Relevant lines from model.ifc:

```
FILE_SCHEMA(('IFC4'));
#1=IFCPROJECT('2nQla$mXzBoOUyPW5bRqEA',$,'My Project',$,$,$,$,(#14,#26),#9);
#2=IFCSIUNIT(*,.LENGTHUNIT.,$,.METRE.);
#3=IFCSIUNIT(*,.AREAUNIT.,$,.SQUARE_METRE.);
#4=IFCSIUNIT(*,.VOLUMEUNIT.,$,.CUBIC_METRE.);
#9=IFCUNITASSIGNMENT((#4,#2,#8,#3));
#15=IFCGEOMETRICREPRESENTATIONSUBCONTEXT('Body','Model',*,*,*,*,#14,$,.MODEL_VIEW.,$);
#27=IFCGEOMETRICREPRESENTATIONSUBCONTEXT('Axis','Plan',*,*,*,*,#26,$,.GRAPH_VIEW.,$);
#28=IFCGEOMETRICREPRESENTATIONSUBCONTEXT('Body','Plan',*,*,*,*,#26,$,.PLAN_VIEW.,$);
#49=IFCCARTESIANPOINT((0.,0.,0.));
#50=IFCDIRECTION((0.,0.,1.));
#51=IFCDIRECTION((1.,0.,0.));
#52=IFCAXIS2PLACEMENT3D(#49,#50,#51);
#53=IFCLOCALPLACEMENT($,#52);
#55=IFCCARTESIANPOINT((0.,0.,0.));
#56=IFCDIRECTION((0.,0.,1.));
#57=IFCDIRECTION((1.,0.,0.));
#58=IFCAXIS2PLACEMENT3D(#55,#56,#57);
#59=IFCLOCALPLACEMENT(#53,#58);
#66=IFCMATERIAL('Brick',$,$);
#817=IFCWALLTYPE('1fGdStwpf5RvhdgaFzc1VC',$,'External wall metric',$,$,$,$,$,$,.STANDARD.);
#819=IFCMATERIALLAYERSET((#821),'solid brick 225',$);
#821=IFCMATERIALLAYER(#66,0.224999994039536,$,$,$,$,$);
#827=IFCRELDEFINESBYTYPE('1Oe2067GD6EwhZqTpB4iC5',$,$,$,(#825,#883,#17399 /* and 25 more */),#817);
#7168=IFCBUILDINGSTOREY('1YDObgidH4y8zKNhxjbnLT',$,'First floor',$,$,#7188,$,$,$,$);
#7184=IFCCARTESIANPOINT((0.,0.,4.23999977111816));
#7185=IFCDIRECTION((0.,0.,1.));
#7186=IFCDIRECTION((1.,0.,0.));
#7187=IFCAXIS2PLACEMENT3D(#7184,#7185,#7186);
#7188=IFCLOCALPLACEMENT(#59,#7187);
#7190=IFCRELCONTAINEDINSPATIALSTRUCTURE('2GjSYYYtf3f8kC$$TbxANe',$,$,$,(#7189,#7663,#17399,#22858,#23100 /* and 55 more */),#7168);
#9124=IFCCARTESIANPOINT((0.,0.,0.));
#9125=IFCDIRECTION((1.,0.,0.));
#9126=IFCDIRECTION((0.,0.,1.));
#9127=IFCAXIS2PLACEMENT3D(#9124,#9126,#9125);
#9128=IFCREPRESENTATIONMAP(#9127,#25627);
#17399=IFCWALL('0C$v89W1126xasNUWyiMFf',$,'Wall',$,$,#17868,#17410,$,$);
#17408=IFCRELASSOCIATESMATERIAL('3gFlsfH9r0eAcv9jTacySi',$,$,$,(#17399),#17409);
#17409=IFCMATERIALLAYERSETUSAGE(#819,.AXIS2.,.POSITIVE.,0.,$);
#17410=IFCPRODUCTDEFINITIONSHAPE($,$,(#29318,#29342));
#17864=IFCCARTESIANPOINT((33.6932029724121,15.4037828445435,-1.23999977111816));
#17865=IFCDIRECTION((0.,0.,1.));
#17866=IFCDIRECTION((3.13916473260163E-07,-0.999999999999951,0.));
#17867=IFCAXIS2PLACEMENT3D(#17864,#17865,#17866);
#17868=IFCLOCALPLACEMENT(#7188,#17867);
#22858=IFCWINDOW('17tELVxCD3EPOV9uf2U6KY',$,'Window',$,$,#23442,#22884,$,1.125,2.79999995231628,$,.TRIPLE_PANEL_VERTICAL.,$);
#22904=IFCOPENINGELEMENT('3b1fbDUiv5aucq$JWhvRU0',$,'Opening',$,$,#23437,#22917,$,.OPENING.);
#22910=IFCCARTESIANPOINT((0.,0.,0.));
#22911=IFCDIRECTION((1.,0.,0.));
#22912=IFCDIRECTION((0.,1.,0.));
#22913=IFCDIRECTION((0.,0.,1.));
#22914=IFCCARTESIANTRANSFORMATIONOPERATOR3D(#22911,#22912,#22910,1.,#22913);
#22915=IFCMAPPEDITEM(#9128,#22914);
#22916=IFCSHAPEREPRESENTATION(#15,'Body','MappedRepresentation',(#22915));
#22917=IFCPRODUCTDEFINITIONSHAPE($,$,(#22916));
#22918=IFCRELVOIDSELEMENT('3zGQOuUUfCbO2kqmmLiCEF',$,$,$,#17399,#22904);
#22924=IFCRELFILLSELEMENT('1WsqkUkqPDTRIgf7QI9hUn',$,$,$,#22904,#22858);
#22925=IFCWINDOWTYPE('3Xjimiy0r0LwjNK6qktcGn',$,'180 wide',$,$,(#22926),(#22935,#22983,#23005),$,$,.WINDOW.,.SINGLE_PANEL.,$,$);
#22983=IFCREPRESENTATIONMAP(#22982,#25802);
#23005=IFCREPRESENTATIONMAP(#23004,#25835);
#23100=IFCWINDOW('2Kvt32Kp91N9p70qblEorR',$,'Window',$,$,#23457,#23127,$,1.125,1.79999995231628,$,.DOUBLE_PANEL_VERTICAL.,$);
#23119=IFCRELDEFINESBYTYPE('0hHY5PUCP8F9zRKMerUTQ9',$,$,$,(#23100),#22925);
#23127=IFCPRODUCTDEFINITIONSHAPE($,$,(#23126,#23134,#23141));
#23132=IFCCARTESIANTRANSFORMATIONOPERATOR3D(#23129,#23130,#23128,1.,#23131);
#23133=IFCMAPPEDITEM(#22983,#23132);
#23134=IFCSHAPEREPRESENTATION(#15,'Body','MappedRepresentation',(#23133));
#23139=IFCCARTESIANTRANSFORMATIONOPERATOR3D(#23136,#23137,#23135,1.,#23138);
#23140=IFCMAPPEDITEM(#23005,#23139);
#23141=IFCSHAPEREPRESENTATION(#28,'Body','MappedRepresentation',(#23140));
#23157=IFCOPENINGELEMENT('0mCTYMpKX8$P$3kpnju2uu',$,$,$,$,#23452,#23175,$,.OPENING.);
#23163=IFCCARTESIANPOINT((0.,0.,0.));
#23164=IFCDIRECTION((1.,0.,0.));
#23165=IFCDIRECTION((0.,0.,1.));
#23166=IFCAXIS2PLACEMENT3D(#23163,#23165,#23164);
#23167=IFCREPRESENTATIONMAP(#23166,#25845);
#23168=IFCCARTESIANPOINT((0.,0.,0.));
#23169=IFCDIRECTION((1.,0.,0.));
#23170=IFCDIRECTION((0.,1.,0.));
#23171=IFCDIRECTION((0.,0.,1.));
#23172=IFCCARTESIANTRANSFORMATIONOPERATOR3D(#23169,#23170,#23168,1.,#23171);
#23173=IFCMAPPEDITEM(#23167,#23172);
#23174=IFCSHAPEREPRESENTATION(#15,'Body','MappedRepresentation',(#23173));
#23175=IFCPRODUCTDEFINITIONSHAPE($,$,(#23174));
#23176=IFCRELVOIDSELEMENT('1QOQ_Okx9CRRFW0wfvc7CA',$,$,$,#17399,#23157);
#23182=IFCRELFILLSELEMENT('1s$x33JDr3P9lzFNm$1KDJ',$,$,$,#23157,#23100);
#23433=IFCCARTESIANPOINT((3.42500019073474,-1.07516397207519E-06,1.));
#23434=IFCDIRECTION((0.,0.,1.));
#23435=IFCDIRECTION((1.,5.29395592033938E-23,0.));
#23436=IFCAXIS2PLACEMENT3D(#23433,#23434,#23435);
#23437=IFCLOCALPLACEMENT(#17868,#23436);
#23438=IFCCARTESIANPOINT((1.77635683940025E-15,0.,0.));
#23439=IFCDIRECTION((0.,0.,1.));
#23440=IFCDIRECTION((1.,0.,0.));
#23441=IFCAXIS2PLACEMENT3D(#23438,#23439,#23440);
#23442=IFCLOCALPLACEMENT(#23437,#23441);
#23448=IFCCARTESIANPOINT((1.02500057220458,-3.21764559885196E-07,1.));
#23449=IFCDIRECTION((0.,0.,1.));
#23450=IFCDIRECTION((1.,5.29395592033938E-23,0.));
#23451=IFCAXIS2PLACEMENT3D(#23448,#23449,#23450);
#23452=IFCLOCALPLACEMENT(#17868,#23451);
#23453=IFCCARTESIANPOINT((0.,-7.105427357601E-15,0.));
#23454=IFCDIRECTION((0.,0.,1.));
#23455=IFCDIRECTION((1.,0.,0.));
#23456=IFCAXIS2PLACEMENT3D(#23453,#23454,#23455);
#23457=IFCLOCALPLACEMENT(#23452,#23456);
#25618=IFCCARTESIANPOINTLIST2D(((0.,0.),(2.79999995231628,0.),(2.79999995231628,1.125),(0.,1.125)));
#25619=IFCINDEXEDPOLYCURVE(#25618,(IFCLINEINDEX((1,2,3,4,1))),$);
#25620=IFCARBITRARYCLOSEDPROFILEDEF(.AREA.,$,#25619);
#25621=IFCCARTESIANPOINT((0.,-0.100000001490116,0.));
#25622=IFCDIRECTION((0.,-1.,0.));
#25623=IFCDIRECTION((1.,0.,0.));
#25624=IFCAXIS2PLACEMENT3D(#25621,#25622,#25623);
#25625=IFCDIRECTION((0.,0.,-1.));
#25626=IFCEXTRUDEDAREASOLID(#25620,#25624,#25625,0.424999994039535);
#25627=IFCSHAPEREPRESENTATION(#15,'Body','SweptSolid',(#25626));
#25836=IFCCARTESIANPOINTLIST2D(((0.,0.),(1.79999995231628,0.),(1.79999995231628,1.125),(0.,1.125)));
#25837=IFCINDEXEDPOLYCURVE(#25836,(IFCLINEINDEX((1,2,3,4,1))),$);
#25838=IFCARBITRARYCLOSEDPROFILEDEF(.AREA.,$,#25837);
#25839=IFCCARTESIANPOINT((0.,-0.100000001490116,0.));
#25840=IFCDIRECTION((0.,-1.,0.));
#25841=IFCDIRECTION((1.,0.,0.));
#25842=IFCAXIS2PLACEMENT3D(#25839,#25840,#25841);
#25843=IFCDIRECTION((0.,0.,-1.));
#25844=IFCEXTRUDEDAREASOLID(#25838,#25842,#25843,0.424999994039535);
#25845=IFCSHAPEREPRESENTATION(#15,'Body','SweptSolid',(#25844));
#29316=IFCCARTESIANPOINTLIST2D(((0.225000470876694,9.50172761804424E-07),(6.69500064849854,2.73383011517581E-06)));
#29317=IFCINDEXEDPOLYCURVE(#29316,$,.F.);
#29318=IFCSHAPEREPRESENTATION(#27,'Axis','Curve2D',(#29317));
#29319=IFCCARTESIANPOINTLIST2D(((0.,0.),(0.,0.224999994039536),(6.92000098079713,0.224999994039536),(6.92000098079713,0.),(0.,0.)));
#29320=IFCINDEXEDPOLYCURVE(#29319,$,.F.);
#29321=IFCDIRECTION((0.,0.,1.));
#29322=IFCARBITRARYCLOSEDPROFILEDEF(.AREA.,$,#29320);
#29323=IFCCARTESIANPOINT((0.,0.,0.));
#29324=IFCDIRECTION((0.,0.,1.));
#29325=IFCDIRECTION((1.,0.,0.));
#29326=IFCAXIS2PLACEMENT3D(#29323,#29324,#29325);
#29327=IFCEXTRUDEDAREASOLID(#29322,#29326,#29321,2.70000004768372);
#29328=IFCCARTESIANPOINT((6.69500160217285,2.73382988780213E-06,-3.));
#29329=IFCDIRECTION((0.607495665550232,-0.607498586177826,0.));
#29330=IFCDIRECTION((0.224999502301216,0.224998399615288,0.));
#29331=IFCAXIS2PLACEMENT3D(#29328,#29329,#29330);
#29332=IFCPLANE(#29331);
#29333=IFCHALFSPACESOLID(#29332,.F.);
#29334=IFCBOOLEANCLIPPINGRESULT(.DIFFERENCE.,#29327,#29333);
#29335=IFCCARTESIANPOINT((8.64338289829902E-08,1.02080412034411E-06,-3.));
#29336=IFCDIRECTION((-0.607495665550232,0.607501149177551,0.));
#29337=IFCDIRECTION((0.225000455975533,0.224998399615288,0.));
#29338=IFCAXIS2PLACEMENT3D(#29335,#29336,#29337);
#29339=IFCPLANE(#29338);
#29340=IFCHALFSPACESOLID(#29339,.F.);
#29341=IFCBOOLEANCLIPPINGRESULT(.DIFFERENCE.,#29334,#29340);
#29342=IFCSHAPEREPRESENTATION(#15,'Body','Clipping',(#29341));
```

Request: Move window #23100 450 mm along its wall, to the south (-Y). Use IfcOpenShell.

```python
import ifcopenshell
import ifcopenshell.api.geometry
import ifcopenshell.util.placement

model = ifcopenshell.open("model.ifc")

window = model.by_guid("2Kvt32Kp91N9p70qblEorR")
opening = window.FillsVoids[0].RelatingOpeningElement
wall = opening.VoidsElements[0].RelatingBuildingElement

wall_matrix = ifcopenshell.util.placement.get_local_placement(wall.ObjectPlacement)
shift = wall_matrix[:3, 0] * 0.45
before = ifcopenshell.util.placement.get_local_placement(window.ObjectPlacement)[:3, 3].copy()

# The window is placed relative to its opening, so it follows when the opening moves.
matrix = ifcopenshell.util.placement.get_local_placement(opening.ObjectPlacement)
matrix[:3, 3] += shift
ifcopenshell.api.geometry.edit_object_placement(
    model, product=opening, matrix=matrix, is_si=False, should_transform_children=True
)

after = ifcopenshell.util.placement.get_local_placement(window.ObjectPlacement)[:3, 3]
print("window moved by", (after - before).round(3) + 0.0)

model.write("model_edited.ifc")
```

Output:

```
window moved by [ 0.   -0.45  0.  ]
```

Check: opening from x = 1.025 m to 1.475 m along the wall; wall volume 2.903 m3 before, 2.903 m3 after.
